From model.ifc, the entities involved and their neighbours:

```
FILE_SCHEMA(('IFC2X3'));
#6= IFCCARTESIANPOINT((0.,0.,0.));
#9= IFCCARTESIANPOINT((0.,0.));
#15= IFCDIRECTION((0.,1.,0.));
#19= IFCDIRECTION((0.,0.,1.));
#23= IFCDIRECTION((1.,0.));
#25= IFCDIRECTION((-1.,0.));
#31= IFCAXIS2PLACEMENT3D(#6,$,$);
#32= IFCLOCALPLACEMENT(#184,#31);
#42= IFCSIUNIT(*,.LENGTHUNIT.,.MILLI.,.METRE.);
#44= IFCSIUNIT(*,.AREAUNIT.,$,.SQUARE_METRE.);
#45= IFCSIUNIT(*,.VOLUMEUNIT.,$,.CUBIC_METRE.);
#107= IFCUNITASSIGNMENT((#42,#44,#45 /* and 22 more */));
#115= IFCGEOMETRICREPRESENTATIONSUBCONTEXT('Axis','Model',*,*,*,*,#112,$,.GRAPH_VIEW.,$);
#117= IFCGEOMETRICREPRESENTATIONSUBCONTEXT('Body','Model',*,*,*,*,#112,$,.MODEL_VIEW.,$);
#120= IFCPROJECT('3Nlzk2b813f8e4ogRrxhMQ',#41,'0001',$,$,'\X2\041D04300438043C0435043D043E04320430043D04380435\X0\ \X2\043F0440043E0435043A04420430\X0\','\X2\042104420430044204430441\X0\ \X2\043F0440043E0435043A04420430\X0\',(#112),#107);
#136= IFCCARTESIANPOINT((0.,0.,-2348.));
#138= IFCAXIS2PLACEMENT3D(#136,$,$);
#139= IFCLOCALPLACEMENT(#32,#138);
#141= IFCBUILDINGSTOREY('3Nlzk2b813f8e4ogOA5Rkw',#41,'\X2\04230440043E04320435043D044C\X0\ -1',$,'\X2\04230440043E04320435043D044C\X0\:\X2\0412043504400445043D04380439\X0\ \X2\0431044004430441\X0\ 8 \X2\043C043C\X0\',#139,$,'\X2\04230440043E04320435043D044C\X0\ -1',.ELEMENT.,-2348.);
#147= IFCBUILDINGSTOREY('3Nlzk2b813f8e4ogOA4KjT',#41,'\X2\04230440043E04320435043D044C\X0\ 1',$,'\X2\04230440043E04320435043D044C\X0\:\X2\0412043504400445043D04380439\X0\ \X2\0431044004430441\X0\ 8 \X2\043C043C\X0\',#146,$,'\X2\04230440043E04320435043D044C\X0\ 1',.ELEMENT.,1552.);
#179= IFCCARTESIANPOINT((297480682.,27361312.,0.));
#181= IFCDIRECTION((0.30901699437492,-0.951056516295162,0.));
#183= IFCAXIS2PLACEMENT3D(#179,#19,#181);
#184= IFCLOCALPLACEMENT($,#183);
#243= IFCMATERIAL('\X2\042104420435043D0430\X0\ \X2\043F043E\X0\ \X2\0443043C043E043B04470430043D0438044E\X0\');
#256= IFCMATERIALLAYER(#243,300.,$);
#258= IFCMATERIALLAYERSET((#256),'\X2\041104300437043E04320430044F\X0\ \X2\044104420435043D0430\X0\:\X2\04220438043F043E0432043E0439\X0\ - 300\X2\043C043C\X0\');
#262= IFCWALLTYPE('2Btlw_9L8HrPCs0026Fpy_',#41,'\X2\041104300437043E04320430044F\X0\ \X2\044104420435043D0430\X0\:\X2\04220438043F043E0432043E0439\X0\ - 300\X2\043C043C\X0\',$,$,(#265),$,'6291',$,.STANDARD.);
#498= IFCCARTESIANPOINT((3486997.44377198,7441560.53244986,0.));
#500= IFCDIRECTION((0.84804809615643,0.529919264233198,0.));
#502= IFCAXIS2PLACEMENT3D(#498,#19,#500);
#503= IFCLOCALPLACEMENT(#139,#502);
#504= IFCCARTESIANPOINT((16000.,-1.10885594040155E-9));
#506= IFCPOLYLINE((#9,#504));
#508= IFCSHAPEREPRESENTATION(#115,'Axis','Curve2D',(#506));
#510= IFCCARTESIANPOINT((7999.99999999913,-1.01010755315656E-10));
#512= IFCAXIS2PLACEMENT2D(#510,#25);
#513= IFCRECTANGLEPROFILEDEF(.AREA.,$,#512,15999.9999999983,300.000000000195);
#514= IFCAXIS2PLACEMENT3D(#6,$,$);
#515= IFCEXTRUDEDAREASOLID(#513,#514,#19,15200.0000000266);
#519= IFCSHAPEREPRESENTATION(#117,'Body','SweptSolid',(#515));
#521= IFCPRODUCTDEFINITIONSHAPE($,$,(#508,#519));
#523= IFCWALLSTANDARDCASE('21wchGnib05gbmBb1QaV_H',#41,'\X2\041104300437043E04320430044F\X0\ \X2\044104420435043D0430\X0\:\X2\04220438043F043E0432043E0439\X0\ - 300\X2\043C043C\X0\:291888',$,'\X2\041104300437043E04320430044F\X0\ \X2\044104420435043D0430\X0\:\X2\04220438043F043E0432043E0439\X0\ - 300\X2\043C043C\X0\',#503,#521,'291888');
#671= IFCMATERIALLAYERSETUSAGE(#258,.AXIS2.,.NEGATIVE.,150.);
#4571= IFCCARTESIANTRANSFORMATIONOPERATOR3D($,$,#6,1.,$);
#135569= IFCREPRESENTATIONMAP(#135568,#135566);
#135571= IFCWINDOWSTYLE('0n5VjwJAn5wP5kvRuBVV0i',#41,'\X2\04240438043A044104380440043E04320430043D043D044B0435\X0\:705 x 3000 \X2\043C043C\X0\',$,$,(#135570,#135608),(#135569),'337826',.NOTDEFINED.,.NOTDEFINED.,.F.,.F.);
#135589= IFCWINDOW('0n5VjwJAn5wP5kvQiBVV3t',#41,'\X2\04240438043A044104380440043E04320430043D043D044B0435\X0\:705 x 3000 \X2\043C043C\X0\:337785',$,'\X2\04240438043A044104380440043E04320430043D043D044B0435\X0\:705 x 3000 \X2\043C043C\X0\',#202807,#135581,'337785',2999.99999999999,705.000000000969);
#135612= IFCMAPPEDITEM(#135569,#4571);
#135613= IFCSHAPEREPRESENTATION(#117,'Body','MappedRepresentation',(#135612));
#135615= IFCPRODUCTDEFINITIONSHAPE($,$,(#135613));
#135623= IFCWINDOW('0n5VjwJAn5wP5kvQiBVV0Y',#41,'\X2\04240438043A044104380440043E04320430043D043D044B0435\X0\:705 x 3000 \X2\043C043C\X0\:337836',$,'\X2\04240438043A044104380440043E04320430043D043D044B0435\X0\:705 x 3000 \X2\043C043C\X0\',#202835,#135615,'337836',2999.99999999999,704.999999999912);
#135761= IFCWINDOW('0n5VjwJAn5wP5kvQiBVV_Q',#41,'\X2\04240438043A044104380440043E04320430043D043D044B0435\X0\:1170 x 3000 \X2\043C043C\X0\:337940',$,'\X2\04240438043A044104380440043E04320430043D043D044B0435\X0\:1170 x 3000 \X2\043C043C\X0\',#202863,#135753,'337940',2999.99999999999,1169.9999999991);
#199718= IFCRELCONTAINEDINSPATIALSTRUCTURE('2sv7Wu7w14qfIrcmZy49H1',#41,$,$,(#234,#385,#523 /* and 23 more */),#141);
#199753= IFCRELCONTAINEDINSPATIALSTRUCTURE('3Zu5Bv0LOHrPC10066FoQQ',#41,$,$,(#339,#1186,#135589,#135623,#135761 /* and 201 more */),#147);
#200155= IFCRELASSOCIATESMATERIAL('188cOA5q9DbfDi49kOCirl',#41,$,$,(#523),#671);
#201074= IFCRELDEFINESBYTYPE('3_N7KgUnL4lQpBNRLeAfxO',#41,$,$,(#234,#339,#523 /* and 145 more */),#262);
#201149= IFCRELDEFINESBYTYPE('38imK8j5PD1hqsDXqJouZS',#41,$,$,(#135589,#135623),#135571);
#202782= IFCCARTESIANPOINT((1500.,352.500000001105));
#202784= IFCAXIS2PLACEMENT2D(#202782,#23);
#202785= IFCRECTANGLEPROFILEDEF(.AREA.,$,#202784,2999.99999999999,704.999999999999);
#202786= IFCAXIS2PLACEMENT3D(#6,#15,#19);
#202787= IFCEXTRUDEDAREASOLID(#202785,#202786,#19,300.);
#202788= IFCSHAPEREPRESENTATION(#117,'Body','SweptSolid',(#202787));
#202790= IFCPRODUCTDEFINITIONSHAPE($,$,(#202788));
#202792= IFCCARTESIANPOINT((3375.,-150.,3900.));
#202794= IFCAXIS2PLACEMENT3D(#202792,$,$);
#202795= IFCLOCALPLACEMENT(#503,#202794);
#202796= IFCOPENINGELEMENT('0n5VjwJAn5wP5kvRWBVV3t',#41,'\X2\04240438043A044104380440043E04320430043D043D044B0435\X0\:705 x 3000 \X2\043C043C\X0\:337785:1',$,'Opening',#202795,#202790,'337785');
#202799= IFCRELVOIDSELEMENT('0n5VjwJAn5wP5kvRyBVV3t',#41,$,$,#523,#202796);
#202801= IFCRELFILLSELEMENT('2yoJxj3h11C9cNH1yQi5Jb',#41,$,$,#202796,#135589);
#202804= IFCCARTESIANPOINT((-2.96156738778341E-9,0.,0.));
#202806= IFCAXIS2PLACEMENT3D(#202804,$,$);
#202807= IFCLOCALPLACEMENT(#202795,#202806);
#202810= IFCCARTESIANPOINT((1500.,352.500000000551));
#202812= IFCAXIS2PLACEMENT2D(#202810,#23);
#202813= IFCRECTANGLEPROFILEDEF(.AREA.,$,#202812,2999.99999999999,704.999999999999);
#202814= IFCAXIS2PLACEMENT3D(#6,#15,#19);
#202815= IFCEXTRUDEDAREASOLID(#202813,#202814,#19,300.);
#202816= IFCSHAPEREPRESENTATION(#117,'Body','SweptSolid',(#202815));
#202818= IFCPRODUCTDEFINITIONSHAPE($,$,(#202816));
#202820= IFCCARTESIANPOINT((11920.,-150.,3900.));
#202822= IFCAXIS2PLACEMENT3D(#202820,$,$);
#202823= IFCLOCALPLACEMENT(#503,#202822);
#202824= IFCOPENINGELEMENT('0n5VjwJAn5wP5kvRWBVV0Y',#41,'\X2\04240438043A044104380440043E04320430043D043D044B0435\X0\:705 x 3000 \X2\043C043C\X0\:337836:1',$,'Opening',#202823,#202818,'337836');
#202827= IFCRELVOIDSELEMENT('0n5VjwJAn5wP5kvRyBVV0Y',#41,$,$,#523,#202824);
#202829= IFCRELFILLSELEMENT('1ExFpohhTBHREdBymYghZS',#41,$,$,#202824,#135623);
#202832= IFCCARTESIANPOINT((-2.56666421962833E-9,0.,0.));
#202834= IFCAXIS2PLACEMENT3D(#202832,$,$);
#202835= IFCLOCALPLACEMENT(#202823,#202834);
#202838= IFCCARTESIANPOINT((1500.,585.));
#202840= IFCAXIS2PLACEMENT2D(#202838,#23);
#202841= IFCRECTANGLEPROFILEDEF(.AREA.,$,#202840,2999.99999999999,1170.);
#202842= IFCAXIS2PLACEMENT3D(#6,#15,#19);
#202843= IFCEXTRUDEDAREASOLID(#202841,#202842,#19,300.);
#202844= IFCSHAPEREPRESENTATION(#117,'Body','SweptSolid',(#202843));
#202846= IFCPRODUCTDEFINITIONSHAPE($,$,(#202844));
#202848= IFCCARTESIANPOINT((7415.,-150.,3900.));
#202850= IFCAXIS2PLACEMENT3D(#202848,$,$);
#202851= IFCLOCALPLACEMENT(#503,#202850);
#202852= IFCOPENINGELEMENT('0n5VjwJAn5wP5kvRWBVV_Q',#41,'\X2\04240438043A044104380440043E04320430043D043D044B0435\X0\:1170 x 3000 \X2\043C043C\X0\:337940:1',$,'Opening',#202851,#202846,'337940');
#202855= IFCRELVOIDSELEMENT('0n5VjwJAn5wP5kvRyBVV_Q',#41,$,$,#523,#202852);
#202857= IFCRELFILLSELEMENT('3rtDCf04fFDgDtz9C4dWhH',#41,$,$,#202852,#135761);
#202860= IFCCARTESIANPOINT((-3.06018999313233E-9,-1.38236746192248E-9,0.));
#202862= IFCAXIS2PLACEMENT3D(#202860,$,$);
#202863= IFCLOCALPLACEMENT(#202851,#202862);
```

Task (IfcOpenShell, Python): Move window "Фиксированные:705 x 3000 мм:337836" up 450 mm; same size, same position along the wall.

```python
import numpy as np
import ifcopenshell
import ifcopenshell.api.geometry
import ifcopenshell.util.placement
import ifcopenshell.util.unit

model = ifcopenshell.open("model.ifc")
unit_scale = ifcopenshell.util.unit.calculate_unit_scale(model)

window = model.by_guid("0n5VjwJAn5wP5kvQiBVV0Y")
opening = window.FillsVoids[0].RelatingOpeningElement
dz = 0.45 / unit_scale

shift = np.array([0.0, 0.0, dz])
# The window is placed relative to its opening, so it follows when the opening moves.
matrix = ifcopenshell.util.placement.get_local_placement(opening.ObjectPlacement)
matrix[:3, 3] += shift
ifcopenshell.api.geometry.edit_object_placement(
    model, product=opening, matrix=matrix, is_si=False, should_transform_children=True
)

print(f"moved by {dz * unit_scale:+.3f} m")

model.write("model-out.ifc")
```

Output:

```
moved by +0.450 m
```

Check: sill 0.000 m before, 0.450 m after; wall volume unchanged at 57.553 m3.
